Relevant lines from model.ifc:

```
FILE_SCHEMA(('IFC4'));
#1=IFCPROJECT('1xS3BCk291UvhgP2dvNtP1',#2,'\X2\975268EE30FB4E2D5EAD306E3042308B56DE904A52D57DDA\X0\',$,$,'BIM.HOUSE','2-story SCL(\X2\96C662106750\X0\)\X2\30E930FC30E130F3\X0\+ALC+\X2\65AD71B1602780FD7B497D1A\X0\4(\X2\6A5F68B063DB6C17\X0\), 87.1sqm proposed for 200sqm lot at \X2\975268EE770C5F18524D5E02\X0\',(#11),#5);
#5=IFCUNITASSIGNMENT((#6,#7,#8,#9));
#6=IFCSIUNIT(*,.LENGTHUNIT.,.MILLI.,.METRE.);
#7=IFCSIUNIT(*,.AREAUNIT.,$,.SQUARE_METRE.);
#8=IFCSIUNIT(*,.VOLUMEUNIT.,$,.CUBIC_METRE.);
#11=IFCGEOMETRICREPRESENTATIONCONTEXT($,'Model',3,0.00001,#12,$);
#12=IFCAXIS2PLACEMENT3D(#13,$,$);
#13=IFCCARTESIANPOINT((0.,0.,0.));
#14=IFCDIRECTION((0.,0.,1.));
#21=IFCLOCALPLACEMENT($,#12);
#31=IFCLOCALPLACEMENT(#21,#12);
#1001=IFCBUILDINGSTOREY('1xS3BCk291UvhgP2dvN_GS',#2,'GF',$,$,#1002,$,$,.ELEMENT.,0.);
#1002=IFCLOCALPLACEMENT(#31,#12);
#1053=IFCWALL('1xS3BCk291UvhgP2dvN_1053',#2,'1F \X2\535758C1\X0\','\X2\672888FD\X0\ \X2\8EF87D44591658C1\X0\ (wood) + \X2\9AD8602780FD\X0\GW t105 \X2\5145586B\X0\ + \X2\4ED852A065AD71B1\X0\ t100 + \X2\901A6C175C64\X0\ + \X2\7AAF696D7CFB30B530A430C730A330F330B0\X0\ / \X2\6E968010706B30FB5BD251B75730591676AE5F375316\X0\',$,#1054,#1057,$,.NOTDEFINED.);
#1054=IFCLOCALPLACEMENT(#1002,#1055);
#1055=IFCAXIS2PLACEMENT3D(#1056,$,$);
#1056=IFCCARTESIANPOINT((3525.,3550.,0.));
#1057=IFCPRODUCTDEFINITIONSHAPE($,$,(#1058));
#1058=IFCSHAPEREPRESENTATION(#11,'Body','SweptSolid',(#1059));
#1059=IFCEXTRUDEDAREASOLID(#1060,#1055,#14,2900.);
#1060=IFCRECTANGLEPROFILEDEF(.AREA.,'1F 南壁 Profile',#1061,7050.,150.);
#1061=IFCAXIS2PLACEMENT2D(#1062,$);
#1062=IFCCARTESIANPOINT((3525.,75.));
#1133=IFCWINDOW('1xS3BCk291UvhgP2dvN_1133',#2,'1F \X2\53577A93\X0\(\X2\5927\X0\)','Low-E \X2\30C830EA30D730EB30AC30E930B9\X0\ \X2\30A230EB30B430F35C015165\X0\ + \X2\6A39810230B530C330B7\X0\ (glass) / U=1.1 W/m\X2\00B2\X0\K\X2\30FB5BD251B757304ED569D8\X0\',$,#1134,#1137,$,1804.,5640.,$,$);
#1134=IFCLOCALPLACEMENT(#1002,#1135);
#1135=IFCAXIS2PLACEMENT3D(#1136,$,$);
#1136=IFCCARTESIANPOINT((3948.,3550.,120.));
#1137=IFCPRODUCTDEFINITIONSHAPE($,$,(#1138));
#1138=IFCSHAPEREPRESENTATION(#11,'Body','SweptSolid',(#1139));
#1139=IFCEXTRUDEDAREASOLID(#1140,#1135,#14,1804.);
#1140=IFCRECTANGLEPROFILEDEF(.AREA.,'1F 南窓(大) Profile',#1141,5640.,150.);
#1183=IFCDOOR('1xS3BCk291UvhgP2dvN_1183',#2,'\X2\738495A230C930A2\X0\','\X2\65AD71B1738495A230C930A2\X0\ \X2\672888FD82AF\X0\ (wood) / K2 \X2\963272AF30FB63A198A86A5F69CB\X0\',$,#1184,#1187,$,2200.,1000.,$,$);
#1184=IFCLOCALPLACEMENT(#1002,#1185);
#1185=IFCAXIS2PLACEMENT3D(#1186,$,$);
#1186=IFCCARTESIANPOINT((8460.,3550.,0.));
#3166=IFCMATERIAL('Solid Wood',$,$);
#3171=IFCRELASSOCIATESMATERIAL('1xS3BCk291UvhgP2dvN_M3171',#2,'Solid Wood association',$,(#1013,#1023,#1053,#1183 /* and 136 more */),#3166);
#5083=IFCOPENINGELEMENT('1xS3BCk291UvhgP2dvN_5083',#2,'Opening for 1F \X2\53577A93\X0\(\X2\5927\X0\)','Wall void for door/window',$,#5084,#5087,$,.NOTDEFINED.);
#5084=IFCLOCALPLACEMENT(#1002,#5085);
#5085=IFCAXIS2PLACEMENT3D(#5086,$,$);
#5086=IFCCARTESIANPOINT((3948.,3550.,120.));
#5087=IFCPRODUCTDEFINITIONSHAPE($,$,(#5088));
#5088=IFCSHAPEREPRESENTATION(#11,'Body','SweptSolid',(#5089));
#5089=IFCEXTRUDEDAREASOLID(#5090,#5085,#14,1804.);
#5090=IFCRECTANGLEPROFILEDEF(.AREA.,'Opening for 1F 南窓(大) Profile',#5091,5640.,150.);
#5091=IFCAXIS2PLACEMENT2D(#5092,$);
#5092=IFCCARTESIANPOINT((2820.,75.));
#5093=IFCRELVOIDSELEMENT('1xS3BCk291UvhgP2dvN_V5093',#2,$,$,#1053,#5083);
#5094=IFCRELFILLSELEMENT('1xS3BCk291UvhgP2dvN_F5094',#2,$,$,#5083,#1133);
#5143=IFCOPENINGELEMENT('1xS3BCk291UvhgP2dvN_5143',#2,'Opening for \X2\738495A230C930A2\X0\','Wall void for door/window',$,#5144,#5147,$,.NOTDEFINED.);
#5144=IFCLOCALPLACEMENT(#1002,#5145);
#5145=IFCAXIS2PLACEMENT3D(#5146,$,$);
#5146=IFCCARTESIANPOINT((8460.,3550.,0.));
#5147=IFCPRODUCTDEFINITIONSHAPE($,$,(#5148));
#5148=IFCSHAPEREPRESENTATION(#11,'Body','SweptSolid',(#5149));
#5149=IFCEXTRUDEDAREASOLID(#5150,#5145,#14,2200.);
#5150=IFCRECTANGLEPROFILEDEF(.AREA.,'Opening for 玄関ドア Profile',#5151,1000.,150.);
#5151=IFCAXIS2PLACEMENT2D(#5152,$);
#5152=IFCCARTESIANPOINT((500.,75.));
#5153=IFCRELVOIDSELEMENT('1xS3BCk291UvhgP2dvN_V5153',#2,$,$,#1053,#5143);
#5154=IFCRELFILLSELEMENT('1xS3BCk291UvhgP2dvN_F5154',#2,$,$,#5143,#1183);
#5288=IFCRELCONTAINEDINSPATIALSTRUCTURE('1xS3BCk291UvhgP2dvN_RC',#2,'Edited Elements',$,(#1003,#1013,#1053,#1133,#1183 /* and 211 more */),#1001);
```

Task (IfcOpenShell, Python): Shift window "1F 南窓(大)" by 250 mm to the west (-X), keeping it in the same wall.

```python
import ifcopenshell
import ifcopenshell.api.geometry
import ifcopenshell.util.placement
import ifcopenshell.util.unit

model = ifcopenshell.open("model.ifc")
unit_scale = ifcopenshell.util.unit.calculate_unit_scale(model)

window = model.by_guid("1xS3BCk291UvhgP2dvN_1133")
opening = window.FillsVoids[0].RelatingOpeningElement
wall = opening.VoidsElements[0].RelatingBuildingElement

wall_matrix = ifcopenshell.util.placement.get_local_placement(wall.ObjectPlacement)
shift = wall_matrix[:3, 0] * -0.25 / unit_scale
before = ifcopenshell.util.placement.get_local_placement(window.ObjectPlacement)[:3, 3].copy()

# The window is not placed relative to its opening, so move both.
for product in (opening, window):
    matrix = ifcopenshell.util.placement.get_local_placement(product.ObjectPlacement)
    matrix[:3, 3] += shift
    ifcopenshell.api.geometry.edit_object_placement(model, product=product, matrix=matrix, is_si=False)

after = ifcopenshell.util.placement.get_local_placement(window.ObjectPlacement)[:3, 3]
print("window moved by", (after - before).round(3) + 0.0)

model.write("model_v2.ifc")
```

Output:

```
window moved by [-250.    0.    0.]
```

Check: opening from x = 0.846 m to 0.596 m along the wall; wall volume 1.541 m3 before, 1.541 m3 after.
